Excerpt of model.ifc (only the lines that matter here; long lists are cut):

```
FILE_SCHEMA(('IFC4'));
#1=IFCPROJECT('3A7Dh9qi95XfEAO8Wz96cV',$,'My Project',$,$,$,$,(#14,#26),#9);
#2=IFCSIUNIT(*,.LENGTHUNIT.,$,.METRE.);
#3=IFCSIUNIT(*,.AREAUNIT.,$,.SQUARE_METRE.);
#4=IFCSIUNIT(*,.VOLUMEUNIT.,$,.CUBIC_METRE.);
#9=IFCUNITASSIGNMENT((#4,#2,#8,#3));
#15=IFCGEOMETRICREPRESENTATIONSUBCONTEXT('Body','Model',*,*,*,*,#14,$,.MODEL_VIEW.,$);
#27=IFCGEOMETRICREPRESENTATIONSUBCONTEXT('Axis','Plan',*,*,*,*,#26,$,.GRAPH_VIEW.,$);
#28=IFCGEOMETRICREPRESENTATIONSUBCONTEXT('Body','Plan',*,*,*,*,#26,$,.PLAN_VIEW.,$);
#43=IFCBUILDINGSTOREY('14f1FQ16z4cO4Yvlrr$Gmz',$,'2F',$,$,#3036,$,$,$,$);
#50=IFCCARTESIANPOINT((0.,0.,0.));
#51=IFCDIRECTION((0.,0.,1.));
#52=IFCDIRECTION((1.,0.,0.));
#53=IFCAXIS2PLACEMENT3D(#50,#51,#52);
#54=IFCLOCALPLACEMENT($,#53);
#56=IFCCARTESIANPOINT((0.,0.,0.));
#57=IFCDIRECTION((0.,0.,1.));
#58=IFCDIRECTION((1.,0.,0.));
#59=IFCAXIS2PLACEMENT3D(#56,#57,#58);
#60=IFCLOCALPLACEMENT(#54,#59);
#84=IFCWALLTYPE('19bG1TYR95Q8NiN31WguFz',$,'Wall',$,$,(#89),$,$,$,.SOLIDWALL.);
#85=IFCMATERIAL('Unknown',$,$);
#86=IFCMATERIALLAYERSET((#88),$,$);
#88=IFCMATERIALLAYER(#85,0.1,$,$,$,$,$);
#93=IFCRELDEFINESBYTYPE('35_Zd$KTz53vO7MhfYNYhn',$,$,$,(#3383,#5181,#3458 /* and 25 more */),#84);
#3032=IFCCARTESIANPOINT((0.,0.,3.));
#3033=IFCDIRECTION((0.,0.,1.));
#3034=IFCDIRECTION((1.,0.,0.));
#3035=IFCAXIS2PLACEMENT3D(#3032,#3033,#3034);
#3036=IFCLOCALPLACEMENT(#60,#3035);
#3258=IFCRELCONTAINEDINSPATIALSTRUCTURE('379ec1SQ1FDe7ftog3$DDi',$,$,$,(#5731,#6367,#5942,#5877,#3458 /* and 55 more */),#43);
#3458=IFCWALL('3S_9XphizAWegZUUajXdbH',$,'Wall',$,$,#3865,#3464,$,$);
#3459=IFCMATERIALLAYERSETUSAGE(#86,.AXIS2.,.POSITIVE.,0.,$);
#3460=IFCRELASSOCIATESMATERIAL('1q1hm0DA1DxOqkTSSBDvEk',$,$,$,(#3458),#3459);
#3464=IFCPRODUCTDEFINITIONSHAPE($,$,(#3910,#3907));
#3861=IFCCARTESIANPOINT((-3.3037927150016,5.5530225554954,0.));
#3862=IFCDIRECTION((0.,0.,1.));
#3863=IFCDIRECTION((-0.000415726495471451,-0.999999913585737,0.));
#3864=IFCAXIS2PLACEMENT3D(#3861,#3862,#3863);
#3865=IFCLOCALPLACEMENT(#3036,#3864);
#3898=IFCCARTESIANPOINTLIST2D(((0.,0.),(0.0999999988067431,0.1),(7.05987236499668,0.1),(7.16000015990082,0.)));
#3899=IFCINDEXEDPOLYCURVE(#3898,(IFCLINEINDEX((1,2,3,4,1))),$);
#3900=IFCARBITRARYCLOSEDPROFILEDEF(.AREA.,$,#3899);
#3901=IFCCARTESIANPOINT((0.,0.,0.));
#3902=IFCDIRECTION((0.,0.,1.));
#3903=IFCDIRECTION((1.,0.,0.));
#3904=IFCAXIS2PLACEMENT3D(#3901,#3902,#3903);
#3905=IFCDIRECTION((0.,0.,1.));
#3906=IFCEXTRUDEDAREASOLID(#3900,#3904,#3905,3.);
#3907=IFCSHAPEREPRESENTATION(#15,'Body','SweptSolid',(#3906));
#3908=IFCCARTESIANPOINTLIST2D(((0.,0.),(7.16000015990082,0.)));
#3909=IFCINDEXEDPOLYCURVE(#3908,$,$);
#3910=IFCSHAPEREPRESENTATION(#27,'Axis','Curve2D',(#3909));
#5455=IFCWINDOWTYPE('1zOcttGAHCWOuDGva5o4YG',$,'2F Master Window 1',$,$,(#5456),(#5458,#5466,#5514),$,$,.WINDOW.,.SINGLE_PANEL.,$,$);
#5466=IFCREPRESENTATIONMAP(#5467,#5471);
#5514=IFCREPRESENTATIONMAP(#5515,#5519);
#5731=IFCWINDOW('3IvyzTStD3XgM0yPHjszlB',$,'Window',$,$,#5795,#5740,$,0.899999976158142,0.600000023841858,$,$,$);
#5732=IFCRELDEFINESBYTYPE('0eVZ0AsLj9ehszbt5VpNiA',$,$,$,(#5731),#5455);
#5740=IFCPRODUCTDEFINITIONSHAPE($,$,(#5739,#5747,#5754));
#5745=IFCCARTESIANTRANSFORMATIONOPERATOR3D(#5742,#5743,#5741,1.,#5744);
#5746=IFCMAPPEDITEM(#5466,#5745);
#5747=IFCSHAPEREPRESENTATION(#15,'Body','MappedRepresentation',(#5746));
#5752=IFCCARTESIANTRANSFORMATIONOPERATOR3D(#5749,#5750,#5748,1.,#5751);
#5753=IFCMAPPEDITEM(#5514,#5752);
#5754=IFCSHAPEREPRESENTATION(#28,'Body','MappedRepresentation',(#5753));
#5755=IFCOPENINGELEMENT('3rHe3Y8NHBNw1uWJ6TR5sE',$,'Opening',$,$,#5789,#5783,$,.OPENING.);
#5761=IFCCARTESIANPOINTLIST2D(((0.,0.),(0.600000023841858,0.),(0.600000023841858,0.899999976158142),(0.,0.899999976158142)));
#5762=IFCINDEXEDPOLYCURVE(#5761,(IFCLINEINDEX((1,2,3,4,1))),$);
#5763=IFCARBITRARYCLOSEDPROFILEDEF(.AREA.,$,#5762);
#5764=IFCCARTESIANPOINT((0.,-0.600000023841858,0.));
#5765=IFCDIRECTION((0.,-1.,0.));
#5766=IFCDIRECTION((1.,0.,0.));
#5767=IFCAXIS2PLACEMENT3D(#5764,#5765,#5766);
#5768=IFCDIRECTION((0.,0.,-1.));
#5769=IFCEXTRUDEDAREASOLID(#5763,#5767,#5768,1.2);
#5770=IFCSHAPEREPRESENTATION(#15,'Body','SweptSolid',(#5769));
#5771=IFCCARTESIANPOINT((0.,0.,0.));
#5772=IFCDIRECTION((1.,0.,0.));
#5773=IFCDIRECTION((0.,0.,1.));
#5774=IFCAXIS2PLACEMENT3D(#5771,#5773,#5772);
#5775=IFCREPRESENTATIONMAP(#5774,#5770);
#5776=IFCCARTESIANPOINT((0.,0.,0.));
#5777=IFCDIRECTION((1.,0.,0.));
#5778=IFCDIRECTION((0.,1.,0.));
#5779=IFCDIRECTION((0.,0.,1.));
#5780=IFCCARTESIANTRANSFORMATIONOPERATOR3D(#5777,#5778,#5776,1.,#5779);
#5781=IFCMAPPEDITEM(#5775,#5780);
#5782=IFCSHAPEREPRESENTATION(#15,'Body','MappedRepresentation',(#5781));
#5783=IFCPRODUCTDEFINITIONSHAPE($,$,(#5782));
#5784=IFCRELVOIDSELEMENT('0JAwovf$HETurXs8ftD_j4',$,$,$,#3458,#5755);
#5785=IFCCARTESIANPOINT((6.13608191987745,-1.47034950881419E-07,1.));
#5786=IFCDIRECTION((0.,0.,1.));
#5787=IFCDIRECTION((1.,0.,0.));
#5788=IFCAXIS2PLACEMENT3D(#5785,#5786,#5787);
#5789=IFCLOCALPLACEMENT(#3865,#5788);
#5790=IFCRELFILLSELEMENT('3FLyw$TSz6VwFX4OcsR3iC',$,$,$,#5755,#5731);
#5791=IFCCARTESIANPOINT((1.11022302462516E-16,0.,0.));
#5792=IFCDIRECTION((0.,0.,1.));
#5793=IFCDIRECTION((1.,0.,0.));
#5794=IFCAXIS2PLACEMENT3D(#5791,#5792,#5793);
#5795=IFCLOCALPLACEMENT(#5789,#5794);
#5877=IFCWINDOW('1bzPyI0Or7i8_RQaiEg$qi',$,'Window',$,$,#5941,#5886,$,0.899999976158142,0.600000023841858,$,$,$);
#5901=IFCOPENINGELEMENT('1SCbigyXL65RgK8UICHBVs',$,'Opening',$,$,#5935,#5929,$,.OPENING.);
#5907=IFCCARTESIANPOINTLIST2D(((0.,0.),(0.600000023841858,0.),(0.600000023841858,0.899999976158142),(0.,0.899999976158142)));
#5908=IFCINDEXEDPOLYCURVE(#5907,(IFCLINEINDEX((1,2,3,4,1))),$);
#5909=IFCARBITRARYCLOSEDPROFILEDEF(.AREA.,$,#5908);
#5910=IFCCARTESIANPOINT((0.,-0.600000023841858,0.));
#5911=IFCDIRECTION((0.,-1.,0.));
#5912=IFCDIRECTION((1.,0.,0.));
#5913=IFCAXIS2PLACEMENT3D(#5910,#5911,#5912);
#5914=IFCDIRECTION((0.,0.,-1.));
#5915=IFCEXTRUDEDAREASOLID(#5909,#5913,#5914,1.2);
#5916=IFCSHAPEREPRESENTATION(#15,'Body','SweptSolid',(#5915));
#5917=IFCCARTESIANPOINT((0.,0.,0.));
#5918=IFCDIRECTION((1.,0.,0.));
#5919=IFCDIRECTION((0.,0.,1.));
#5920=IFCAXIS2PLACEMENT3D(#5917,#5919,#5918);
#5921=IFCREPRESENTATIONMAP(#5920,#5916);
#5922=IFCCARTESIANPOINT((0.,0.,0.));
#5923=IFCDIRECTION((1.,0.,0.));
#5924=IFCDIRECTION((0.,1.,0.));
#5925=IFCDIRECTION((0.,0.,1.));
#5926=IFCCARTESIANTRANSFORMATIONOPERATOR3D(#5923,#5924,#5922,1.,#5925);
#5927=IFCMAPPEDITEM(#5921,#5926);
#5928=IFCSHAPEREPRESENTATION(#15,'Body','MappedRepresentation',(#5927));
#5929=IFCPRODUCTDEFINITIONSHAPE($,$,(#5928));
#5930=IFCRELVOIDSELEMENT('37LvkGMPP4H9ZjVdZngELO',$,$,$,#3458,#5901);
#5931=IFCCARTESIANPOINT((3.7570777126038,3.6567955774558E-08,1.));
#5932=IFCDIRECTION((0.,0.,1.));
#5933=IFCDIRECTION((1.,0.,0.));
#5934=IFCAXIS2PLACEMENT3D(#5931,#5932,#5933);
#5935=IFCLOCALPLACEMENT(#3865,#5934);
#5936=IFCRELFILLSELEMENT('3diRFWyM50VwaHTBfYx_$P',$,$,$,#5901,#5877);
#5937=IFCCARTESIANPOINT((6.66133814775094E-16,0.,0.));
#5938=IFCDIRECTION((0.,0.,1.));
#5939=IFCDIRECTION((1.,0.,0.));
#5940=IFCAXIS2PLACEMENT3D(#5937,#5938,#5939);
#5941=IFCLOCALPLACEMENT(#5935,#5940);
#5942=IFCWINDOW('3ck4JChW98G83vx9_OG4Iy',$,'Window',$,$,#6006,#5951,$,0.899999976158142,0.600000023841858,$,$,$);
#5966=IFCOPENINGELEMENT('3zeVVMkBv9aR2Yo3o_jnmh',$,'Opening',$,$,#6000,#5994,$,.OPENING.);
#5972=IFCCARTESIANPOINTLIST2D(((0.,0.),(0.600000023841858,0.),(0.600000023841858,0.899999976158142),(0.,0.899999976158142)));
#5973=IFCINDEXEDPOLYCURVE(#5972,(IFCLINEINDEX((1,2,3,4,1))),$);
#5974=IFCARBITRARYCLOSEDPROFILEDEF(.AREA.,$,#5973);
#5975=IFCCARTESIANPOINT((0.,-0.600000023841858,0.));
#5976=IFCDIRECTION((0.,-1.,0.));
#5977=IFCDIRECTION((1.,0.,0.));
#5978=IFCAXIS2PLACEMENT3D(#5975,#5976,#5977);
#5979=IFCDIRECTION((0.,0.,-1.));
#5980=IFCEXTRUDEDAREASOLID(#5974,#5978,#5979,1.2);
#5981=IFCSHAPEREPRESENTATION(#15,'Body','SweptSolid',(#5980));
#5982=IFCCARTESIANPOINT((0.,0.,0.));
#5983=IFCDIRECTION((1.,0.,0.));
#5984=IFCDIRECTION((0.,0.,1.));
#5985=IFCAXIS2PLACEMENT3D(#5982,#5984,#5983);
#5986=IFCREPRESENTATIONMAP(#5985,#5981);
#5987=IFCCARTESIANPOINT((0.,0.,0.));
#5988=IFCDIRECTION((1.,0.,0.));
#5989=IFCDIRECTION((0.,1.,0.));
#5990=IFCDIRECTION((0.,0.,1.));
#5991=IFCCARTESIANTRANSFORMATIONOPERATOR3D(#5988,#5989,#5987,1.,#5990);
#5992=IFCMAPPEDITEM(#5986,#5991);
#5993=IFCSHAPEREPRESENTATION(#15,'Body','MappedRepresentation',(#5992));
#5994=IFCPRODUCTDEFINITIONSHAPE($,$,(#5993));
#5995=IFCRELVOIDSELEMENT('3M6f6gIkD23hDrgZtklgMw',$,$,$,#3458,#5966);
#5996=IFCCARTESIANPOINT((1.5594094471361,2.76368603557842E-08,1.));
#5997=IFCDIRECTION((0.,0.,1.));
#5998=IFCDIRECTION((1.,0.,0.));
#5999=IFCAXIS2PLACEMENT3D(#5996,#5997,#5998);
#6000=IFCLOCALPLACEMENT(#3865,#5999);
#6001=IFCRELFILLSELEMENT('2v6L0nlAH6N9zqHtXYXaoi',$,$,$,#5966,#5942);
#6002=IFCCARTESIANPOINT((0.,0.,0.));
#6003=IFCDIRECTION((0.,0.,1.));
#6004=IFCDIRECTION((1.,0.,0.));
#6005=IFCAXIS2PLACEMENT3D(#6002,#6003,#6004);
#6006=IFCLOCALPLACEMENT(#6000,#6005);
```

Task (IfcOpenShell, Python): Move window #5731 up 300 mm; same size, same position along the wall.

```python
import numpy as np
import ifcopenshell
import ifcopenshell.api.geometry
import ifcopenshell.util.placement
import ifcopenshell.util.unit

model = ifcopenshell.open("model.ifc")
unit_scale = ifcopenshell.util.unit.calculate_unit_scale(model)

window = model.by_guid("3IvyzTStD3XgM0yPHjszlB")
opening = window.FillsVoids[0].RelatingOpeningElement
dz = 0.3 / unit_scale

shift = np.array([0.0, 0.0, dz])
# The window is placed relative to its opening, so it follows when the opening moves.
matrix = ifcopenshell.util.placement.get_local_placement(opening.ObjectPlacement)
matrix[:3, 3] += shift
ifcopenshell.api.geometry.edit_object_placement(
    model, product=opening, matrix=matrix, is_si=False, should_transform_children=True
)

print(f"moved by {dz * unit_scale:+.3f} m")

model.write("model_rev.ifc")
```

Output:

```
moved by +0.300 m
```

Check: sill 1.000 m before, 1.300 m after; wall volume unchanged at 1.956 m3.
